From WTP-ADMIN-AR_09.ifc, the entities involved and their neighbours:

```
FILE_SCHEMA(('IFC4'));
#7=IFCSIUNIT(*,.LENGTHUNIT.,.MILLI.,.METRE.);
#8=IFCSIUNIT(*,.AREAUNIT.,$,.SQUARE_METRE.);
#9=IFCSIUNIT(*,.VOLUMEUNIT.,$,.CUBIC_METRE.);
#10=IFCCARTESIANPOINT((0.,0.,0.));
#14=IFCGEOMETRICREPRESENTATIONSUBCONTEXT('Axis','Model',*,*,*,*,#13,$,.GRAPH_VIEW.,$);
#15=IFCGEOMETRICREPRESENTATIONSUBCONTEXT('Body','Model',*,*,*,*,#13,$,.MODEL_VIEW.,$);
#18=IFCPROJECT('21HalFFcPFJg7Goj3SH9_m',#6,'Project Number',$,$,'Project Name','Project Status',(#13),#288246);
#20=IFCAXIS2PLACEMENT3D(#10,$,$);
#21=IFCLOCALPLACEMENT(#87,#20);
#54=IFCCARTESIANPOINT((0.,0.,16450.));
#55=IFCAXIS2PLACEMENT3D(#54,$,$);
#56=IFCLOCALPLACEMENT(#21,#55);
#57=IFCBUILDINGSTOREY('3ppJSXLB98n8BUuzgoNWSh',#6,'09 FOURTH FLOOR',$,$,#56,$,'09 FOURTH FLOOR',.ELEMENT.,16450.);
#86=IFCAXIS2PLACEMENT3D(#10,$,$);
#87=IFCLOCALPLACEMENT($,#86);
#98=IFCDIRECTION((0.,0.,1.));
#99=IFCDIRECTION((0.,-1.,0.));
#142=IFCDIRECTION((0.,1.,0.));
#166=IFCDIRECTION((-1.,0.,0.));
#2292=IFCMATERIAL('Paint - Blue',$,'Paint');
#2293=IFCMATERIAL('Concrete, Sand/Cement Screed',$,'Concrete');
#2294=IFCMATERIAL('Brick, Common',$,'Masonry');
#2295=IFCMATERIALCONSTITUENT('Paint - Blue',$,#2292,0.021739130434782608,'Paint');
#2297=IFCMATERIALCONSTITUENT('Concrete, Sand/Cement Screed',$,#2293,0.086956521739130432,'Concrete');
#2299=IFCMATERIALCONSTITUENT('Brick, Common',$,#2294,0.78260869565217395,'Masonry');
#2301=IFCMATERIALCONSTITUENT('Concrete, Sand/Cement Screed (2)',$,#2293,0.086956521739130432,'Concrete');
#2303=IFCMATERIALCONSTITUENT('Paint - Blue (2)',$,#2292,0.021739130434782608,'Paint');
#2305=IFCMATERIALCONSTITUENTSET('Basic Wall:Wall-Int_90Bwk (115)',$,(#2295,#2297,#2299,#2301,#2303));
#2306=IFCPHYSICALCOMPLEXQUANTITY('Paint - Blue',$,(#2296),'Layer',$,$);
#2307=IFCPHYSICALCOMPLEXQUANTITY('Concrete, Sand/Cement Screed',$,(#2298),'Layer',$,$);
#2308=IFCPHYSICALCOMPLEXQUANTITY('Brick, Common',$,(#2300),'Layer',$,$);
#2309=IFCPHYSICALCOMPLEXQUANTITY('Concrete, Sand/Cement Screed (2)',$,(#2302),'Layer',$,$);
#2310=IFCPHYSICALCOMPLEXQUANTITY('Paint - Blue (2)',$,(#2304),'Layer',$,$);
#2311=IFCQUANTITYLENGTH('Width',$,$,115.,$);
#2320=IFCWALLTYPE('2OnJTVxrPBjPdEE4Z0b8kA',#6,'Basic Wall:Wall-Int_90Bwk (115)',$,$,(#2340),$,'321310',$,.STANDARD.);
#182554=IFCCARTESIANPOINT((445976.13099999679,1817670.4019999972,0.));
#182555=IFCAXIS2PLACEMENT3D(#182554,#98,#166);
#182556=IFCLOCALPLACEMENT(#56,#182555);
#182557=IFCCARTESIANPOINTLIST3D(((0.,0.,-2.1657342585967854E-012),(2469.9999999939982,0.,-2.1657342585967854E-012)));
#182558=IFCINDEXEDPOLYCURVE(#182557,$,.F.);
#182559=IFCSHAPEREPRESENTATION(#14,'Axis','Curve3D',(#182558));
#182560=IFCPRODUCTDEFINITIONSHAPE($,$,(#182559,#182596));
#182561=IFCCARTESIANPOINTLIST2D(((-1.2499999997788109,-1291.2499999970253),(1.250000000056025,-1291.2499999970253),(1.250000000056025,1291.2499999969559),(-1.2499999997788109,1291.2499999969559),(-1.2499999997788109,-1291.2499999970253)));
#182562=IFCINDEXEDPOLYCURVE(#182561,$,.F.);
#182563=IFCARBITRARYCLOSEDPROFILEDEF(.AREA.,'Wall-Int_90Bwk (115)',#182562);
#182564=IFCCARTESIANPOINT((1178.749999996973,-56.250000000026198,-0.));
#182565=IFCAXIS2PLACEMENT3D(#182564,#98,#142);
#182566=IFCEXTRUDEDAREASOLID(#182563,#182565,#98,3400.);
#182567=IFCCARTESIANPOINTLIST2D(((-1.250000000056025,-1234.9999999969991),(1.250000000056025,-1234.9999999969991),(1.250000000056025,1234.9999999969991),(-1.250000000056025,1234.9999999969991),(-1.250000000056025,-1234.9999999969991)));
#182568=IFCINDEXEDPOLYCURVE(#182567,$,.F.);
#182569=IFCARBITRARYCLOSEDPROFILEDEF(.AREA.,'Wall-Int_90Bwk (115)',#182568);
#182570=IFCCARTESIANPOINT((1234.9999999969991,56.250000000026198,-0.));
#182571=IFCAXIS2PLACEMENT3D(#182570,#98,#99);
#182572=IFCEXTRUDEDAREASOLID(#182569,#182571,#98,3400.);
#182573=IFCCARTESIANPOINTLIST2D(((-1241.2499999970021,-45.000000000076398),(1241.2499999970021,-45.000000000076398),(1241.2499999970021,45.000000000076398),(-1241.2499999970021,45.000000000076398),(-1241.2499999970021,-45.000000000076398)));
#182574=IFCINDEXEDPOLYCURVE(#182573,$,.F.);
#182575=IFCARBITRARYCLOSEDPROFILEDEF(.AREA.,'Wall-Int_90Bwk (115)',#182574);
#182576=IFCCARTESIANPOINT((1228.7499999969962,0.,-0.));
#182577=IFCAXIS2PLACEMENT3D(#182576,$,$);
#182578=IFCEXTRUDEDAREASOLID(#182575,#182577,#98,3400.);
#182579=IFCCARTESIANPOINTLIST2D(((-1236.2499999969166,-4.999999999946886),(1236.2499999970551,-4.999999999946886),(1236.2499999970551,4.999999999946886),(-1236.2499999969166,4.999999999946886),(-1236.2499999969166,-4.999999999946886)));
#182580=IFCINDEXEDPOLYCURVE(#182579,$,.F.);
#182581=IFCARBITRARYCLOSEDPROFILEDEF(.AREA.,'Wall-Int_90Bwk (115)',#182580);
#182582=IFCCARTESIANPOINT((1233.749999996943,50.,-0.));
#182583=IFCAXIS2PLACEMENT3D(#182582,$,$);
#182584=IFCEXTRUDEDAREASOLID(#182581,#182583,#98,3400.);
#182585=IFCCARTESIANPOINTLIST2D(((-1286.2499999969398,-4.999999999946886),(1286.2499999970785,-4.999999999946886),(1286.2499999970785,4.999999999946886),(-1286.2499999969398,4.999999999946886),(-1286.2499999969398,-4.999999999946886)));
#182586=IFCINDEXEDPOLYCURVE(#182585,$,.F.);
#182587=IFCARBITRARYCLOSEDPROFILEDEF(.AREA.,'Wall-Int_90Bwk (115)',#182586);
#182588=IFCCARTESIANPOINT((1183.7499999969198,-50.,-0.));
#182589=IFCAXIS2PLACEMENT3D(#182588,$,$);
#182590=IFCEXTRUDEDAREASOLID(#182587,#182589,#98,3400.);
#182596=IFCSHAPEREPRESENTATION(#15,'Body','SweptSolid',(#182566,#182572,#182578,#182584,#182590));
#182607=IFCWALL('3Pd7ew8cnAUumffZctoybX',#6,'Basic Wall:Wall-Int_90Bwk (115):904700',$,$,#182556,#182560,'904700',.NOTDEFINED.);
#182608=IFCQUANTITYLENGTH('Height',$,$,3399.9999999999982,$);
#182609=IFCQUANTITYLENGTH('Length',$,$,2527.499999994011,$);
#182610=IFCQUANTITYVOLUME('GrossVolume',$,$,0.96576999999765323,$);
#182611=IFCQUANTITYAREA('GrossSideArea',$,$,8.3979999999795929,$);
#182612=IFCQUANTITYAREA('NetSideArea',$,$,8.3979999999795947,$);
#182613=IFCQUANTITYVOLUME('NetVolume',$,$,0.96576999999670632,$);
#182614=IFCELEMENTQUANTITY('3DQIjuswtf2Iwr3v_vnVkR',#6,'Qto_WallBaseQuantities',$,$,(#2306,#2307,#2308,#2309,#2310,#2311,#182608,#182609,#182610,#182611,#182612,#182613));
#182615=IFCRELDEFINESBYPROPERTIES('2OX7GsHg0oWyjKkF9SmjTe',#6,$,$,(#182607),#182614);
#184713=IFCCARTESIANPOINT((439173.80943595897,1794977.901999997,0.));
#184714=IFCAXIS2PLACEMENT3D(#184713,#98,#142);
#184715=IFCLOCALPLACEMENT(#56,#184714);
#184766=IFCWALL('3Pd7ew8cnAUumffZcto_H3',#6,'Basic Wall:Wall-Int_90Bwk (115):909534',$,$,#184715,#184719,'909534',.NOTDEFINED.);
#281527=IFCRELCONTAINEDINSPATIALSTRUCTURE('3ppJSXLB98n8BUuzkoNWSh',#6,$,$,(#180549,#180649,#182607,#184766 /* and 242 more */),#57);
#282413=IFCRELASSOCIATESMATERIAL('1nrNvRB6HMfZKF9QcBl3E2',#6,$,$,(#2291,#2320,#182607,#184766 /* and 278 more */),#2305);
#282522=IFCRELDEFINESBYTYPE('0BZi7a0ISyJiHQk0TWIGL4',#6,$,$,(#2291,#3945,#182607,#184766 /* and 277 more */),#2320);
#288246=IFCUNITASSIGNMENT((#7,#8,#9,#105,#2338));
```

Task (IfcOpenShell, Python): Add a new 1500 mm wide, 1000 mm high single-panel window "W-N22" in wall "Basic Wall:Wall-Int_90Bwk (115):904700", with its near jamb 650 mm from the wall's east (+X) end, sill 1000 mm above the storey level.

```python
import numpy as np
import ifcopenshell
import ifcopenshell.api.feature
import ifcopenshell.api.geometry
import ifcopenshell.api.pset
import ifcopenshell.api.root
import ifcopenshell.api.spatial
import ifcopenshell.geom
import ifcopenshell.util.element
import ifcopenshell.util.placement
import ifcopenshell.util.representation
import ifcopenshell.util.shape
import ifcopenshell.util.unit

model = ifcopenshell.open("WTP-ADMIN-AR_09.ifc")
unit_scale = ifcopenshell.util.unit.calculate_unit_scale(model)
area_scale = ifcopenshell.util.unit.calculate_unit_scale(model, "AREAUNIT")
volume_scale = ifcopenshell.util.unit.calculate_unit_scale(model, "VOLUMEUNIT")
settings = ifcopenshell.geom.settings()


def volume(element):
    """Net volume in cubic metres, openings subtracted."""
    shape = ifcopenshell.geom.create_shape(settings, element)
    return ifcopenshell.util.shape.get_volume(shape.geometry)


wall = model.by_guid("3Pd7ew8cnAUumffZctoybX")
storey = ifcopenshell.util.element.get_container(wall, ifc_class="IfcBuildingStorey")
context = ifcopenshell.util.representation.get_context(model, "Model", "Body", "MODEL_VIEW")
before = volume(wall)

width, height, from_end, sill = 1.5, 1, 0.65, 1  # metres

# The wall runs along its own X axis, and the end named is its -X end.
wall_shape = ifcopenshell.geom.create_shape(settings, wall)
x, y, z = ifcopenshell.util.shape.get_vertices(wall_shape.geometry).T
start = x.min() + from_end
face, thickness = float(y.min()), float(y.max() - y.min())
wall_matrix = ifcopenshell.util.placement.get_local_placement(wall.ObjectPlacement)
level = ifcopenshell.util.placement.get_local_placement(storey.ObjectPlacement)[2, 3]


def in_wall(x, y):
    """Placement at x, y metres in the wall's axes, at sill height."""
    matrix = wall_matrix.copy()
    matrix[:, 3] = wall_matrix @ np.array([x / unit_scale, y / unit_scale, 0.0, 1.0])
    matrix[2, 3] = level + sill / unit_scale
    return matrix


# Opening: a box that overshoots both wall faces by 50 mm.
opening = ifcopenshell.api.root.create_entity(model, ifc_class="IfcOpeningElement", predefined_type="OPENING")
box = ifcopenshell.api.geometry.add_wall_representation(
    model, context=context, length=width, height=height, thickness=thickness + 0.1
)
ifcopenshell.api.geometry.assign_representation(model, product=opening, representation=box)
ifcopenshell.api.geometry.edit_object_placement(model, product=opening, matrix=in_wall(start, face - 0.05), is_si=False)
ifcopenshell.api.feature.add_feature(model, feature=opening, element=wall)

window = ifcopenshell.api.root.create_entity(model, ifc_class="IfcWindow", name="W-N22", predefined_type="WINDOW")
window.OverallWidth, window.OverallHeight = width / unit_scale, height / unit_scale
window.PartitioningType = "SINGLE_PANEL"
body = ifcopenshell.api.geometry.add_window_representation(
    model,
    context=context,
    overall_width=window.OverallWidth,
    overall_height=window.OverallHeight,
    partition_type="SINGLE_PANEL",
)
ifcopenshell.api.geometry.assign_representation(model, product=window, representation=body)
ifcopenshell.api.spatial.assign_container(model, products=[window], relating_structure=storey)
ifcopenshell.api.feature.add_filling(model, opening=opening, element=window)

# Centre the window in the wall's thickness.
ifcopenshell.api.geometry.edit_object_placement(model, product=window, matrix=in_wall(start, face), is_si=False)
window_shape = ifcopenshell.geom.create_shape(settings, window)
depth = ifcopenshell.util.shape.get_vertices(window_shape.geometry)[:, 1]
offset = face + thickness / 2 - (depth.min() + depth.max()) / 2
ifcopenshell.api.geometry.edit_object_placement(model, product=window, matrix=in_wall(start, offset), is_si=False)

after = volume(wall)

# Update the wall's stored quantities.
qto = model.by_id(ifcopenshell.util.element.get_pset(wall, "Qto_WallBaseQuantities", should_inherit=False)["id"])
ifcopenshell.api.pset.edit_qto(model, qto=qto, properties={
    "NetSideArea": after / thickness / area_scale,
    "NetVolume": after / volume_scale,
})

print(f"wall volume {before:.3f} -> {after:.3f} m3")

model.write("WTP-ADMIN-AR_09_updated.ifc")
```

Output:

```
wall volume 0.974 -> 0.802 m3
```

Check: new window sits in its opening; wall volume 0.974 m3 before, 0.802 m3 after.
